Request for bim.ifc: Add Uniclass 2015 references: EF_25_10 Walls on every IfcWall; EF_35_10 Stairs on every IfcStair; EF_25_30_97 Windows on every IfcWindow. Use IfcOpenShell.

First a look at what the model holds.

```python
import ifcopenshell

model = ifcopenshell.open("bim.ifc")
print(model.schema)
print("classifications:", [c.Name for c in model.by_type("IfcClassification")])
for ifc_class in ("IfcDoor", "IfcRoof", "IfcStair", "IfcWall", "IfcWindow"):
    print(ifc_class, len(model.by_type(ifc_class)))
```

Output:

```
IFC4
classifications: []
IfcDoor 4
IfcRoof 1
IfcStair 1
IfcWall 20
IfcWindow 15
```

```python
import ifcopenshell
import ifcopenshell.api.classification

model = ifcopenshell.open("bim.ifc")

system = ifcopenshell.api.classification.add_classification(model, classification="Uniclass 2015")

codes = {
    "IfcWall": ("EF_25_10", "Walls"),
    "IfcStair": ("EF_35_10", "Stairs"),
    "IfcWindow": ("EF_25_30_97", "Windows"),
}
for ifc_class, (code, name) in codes.items():
    products = model.by_type(ifc_class)
    ifcopenshell.api.classification.add_reference(
        model, products=products, classification=system, identification=code, name=name
    )
    print(code, len(products))

model.write("bim_edited.ifc")
```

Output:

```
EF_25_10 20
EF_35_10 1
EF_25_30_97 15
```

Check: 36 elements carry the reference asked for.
